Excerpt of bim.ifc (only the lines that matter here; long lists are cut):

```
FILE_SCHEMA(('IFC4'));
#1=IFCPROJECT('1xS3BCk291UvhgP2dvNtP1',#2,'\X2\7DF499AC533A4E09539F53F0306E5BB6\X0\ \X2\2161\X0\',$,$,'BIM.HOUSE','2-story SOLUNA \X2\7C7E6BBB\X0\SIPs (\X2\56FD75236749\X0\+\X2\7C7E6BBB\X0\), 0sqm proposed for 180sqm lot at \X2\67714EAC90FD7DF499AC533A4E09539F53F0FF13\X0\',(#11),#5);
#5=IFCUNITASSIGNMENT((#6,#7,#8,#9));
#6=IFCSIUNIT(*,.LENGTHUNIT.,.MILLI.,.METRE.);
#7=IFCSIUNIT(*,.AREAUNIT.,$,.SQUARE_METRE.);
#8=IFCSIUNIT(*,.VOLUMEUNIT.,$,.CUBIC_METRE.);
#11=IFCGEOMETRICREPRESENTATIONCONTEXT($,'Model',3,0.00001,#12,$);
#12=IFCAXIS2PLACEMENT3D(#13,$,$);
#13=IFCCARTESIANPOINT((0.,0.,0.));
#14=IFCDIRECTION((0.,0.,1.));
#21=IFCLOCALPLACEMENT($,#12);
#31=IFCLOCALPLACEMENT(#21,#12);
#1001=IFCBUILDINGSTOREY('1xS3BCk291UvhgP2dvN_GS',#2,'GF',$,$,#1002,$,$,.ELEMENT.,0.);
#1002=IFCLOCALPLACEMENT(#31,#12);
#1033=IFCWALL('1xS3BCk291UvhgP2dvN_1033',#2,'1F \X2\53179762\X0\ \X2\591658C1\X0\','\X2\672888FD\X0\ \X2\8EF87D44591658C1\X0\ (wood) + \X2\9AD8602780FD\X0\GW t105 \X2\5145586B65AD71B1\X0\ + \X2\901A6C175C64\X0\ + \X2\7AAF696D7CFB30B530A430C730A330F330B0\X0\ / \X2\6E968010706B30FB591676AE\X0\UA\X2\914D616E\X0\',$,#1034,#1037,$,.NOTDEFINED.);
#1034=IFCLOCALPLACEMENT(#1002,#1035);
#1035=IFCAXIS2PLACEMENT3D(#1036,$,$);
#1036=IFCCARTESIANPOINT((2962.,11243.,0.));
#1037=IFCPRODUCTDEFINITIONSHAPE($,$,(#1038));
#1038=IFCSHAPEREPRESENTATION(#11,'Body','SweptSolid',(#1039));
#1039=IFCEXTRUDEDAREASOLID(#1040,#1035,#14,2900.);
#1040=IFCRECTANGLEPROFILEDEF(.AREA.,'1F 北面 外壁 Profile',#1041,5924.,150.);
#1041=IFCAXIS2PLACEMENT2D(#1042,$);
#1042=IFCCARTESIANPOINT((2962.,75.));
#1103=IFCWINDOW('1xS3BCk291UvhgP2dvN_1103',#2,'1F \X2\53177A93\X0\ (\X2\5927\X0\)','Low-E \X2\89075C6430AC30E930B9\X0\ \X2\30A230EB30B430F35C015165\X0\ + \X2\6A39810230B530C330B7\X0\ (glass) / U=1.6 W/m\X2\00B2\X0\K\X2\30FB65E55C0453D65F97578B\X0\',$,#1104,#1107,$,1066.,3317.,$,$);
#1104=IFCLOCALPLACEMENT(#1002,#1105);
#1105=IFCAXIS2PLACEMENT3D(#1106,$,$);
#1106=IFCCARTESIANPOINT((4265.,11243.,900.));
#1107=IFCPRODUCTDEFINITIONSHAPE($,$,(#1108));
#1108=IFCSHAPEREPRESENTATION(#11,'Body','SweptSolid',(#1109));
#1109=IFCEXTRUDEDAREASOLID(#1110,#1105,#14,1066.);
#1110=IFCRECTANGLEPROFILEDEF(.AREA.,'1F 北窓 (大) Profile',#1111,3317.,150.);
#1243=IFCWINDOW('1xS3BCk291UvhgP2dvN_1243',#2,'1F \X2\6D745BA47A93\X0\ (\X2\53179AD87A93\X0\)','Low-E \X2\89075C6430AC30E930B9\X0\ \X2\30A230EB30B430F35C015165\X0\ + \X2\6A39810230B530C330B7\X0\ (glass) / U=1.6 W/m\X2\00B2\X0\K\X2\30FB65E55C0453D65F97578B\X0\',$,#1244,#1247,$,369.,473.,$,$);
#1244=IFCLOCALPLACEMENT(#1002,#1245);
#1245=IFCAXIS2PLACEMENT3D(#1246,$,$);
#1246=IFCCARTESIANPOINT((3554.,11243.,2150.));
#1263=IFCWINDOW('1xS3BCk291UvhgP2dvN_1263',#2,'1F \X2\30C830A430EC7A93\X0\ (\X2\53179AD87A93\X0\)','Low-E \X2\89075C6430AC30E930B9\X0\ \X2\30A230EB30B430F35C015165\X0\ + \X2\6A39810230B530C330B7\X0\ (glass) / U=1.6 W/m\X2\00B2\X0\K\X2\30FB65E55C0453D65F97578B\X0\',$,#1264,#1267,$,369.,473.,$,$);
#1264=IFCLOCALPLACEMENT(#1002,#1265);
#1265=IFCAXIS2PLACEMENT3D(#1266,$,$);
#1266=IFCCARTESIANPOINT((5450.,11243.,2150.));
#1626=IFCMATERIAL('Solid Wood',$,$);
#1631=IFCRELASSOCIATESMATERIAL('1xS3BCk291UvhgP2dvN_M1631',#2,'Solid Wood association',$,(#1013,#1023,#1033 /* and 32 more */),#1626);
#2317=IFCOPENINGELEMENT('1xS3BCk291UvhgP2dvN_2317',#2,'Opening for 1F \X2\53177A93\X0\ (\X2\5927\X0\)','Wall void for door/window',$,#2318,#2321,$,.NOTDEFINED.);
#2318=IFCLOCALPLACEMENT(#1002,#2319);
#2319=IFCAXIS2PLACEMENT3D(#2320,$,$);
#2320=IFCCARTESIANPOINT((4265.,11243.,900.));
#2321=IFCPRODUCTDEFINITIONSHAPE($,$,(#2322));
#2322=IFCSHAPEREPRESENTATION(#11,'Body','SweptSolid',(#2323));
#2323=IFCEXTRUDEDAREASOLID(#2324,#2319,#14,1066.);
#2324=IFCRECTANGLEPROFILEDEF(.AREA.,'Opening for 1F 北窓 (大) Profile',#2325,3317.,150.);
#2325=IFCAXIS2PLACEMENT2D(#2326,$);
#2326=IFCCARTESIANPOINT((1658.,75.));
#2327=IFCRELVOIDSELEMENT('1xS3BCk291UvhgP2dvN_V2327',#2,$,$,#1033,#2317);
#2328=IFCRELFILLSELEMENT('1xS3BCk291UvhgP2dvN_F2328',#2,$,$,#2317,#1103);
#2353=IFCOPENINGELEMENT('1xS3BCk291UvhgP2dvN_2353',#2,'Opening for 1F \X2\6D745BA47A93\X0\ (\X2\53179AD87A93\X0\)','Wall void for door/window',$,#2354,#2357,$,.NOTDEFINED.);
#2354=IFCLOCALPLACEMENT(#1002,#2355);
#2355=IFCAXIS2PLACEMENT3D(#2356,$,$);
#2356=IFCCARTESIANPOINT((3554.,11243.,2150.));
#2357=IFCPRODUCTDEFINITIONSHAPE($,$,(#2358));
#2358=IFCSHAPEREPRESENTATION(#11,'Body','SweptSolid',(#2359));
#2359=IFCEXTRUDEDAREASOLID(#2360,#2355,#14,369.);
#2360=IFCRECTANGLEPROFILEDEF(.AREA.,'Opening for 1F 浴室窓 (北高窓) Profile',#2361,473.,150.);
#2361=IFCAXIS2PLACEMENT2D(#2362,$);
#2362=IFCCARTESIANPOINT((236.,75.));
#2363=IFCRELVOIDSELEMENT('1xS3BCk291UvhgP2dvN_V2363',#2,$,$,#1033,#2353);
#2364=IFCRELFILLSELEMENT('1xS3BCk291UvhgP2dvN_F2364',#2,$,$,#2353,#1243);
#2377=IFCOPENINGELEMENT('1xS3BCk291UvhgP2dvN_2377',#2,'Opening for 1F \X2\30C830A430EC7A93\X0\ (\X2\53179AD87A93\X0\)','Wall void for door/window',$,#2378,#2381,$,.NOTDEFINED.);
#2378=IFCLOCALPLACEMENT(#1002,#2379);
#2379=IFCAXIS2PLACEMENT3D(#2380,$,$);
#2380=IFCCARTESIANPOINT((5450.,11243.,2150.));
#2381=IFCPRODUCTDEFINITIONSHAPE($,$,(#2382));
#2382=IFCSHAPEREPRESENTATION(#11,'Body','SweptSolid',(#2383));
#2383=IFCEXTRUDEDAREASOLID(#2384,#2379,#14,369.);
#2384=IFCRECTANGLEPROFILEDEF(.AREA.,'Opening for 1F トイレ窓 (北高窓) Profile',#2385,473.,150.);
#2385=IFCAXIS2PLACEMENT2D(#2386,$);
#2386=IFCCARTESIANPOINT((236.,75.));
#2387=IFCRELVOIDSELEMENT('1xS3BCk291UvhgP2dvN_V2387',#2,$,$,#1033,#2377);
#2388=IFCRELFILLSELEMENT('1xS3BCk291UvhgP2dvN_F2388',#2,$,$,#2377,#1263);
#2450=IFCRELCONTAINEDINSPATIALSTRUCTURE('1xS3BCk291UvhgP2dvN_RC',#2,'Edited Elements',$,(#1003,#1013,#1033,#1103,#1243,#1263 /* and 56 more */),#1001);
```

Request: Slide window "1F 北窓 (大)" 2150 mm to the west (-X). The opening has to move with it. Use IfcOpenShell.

```python
import ifcopenshell
import ifcopenshell.api.geometry
import ifcopenshell.util.placement
import ifcopenshell.util.unit

model = ifcopenshell.open("bim.ifc")
unit_scale = ifcopenshell.util.unit.calculate_unit_scale(model)

window = model.by_guid("1xS3BCk291UvhgP2dvN_1103")
opening = window.FillsVoids[0].RelatingOpeningElement
wall = opening.VoidsElements[0].RelatingBuildingElement

wall_matrix = ifcopenshell.util.placement.get_local_placement(wall.ObjectPlacement)
shift = wall_matrix[:3, 0] * -2.15 / unit_scale
before = ifcopenshell.util.placement.get_local_placement(window.ObjectPlacement)[:3, 3].copy()

# The window is not placed relative to its opening, so move both.
for product in (opening, window):
    matrix = ifcopenshell.util.placement.get_local_placement(product.ObjectPlacement)
    matrix[:3, 3] += shift
    ifcopenshell.api.geometry.edit_object_placement(model, product=product, matrix=matrix, is_si=False)

after = ifcopenshell.util.placement.get_local_placement(window.ObjectPlacement)[:3, 3]
print("window moved by", (after - before).round(3) + 0.0)

model.write("bim-out.ifc")
```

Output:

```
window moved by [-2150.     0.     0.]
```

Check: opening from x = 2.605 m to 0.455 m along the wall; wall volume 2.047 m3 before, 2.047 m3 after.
